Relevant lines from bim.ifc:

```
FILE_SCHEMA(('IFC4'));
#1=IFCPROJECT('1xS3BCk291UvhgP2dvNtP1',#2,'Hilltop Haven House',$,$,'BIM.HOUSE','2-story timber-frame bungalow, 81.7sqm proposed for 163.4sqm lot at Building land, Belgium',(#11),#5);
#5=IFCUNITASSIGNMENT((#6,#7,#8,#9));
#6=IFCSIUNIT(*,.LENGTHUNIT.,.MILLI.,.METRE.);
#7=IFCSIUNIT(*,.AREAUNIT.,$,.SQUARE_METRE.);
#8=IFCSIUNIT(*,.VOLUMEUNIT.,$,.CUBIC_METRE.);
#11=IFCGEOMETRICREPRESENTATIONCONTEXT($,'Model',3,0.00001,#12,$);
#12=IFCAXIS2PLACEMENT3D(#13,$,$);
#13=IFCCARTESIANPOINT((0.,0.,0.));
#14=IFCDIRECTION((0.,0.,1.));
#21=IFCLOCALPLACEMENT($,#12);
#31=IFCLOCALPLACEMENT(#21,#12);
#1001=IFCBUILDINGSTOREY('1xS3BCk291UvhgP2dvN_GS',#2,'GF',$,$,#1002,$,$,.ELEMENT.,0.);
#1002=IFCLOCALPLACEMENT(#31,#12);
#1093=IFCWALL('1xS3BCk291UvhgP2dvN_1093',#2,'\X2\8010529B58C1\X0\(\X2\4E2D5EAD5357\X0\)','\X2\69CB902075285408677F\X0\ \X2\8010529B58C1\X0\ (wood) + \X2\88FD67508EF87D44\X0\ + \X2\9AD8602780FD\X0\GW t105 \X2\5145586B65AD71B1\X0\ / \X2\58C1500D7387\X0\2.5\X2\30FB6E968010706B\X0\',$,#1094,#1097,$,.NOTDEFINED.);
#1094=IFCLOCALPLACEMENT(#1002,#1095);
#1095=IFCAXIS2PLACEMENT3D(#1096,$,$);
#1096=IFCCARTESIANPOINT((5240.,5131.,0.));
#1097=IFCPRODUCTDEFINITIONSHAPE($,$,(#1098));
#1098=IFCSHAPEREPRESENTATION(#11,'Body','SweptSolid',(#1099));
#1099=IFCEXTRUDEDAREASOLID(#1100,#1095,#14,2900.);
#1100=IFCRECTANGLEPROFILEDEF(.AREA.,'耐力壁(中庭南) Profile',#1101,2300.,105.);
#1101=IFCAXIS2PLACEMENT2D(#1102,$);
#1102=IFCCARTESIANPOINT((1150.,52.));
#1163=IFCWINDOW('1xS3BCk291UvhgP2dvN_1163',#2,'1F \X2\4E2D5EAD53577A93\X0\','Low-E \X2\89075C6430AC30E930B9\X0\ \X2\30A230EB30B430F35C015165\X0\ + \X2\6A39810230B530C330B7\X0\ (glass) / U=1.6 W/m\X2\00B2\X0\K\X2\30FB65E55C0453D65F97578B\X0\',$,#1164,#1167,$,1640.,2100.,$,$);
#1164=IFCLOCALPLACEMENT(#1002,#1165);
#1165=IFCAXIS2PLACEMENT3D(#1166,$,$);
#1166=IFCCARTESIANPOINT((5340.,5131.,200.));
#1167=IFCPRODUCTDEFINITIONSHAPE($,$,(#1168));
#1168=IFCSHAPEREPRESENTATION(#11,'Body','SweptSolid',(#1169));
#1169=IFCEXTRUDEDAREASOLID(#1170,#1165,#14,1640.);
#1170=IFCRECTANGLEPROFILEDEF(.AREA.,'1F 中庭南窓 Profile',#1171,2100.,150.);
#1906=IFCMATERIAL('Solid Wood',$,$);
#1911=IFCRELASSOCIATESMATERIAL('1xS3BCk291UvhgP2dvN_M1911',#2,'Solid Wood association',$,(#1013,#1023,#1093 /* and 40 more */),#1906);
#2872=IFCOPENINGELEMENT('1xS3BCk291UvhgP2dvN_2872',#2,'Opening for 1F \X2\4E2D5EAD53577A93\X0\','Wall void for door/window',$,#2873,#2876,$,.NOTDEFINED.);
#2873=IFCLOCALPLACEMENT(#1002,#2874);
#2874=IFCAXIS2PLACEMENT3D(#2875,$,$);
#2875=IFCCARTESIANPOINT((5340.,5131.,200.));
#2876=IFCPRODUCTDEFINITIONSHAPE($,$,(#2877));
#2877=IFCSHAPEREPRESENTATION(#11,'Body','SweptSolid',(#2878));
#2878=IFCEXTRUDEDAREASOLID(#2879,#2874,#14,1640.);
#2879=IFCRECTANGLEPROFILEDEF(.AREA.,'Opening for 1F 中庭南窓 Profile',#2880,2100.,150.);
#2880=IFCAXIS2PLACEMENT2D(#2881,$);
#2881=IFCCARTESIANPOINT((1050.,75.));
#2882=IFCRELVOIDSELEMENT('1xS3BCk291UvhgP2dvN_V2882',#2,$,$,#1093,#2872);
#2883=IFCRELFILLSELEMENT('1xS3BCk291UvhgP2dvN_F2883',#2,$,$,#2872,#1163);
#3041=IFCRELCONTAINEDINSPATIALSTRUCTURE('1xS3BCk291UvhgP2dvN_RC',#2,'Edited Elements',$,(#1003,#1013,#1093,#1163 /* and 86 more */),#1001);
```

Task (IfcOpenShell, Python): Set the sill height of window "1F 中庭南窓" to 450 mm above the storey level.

```python
import numpy as np
import ifcopenshell
import ifcopenshell.api.geometry
import ifcopenshell.geom
import ifcopenshell.util.element
import ifcopenshell.util.placement
import ifcopenshell.util.shape
import ifcopenshell.util.unit

model = ifcopenshell.open("bim.ifc")
unit_scale = ifcopenshell.util.unit.calculate_unit_scale(model)

window = model.by_id(1163)
opening = window.FillsVoids[0].RelatingOpeningElement
storey = ifcopenshell.util.element.get_container(window, ifc_class="IfcBuildingStorey")
level = ifcopenshell.util.placement.get_local_placement(storey.ObjectPlacement)[2, 3]

# The opening's origin need not be at the sill, so measure its lowest point.
shape = ifcopenshell.geom.create_shape(ifcopenshell.geom.settings(), opening)
bottom = ifcopenshell.util.shape.get_shape_bottom_elevation(shape, shape.geometry) / unit_scale
dz = level + 0.45 / unit_scale - bottom

shift = np.array([0.0, 0.0, dz])
# The window is not placed relative to its opening, so move both.
for product in (opening, window):
    matrix = ifcopenshell.util.placement.get_local_placement(product.ObjectPlacement)
    matrix[:3, 3] += shift
    ifcopenshell.api.geometry.edit_object_placement(model, product=product, matrix=matrix, is_si=False)

print(f"moved by {dz * unit_scale:+.3f} m")

model.write("bim-out.ifc")
```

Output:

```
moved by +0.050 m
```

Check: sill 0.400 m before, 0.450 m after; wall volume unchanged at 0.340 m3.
